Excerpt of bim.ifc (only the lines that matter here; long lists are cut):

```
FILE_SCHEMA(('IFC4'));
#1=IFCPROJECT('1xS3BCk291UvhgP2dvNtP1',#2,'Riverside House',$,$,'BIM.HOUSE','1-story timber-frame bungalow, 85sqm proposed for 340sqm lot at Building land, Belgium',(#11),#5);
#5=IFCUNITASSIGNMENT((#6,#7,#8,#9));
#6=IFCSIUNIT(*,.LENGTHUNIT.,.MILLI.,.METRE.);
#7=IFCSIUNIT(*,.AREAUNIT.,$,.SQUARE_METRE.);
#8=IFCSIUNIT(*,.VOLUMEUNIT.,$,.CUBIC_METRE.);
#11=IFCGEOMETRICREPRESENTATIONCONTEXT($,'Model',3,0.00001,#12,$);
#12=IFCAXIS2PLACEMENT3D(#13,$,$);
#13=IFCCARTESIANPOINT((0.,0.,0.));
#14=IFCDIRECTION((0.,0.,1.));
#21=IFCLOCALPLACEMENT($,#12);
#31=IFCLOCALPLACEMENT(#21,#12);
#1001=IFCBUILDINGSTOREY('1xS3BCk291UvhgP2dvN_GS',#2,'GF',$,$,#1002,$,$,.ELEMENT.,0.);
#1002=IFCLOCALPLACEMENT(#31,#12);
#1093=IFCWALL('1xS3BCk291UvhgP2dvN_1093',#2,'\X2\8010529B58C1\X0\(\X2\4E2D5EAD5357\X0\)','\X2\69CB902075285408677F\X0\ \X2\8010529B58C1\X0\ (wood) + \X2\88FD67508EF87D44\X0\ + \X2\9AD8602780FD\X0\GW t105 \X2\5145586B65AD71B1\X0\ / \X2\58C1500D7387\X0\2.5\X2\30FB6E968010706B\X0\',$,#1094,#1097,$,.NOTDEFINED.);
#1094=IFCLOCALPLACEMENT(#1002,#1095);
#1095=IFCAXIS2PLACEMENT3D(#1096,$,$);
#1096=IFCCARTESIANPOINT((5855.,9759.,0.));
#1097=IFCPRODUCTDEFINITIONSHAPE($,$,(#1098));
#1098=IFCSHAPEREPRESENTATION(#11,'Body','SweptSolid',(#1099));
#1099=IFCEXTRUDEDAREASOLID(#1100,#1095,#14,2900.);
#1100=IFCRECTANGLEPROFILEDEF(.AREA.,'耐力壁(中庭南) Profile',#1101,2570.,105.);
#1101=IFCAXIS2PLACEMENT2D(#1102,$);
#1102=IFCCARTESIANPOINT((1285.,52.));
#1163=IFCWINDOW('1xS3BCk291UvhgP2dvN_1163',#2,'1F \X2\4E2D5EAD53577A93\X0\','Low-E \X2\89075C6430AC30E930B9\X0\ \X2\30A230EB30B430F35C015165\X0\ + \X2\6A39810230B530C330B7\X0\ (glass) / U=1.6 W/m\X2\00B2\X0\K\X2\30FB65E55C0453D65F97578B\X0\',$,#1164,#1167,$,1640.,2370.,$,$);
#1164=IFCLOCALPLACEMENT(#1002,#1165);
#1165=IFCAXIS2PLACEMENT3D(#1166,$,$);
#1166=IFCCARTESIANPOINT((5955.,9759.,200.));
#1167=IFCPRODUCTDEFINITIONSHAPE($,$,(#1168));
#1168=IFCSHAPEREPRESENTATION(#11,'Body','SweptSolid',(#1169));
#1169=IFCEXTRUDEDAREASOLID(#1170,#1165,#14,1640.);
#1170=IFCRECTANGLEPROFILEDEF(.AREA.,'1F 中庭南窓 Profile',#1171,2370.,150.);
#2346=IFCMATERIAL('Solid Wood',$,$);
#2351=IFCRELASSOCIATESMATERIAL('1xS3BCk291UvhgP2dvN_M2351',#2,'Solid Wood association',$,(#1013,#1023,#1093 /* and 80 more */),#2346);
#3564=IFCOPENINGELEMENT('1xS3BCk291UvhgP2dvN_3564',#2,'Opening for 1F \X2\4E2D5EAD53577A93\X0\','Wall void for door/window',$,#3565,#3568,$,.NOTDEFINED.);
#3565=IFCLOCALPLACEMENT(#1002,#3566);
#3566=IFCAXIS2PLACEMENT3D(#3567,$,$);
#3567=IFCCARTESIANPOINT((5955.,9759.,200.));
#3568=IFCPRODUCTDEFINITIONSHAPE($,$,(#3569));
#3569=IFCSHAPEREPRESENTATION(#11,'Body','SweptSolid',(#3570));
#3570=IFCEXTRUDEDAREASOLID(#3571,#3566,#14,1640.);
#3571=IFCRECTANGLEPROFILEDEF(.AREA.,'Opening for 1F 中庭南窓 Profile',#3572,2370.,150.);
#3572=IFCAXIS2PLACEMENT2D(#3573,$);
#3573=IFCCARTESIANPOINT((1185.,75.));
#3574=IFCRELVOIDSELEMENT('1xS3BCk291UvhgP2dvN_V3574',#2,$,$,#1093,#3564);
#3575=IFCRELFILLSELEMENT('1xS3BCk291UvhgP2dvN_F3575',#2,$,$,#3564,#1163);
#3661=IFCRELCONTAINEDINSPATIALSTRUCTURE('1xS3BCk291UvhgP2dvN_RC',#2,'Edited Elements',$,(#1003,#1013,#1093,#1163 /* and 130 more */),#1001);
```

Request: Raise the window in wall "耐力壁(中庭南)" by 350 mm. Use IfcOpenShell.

```python
import numpy as np
import ifcopenshell
import ifcopenshell.api.geometry
import ifcopenshell.util.placement
import ifcopenshell.util.unit

model = ifcopenshell.open("bim.ifc")
unit_scale = ifcopenshell.util.unit.calculate_unit_scale(model)

window = model.by_guid("1xS3BCk291UvhgP2dvN_1163")
opening = window.FillsVoids[0].RelatingOpeningElement
dz = 0.35 / unit_scale

shift = np.array([0.0, 0.0, dz])
# The window is not placed relative to its opening, so move both.
for product in (opening, window):
    matrix = ifcopenshell.util.placement.get_local_placement(product.ObjectPlacement)
    matrix[:3, 3] += shift
    ifcopenshell.api.geometry.edit_object_placement(model, product=product, matrix=matrix, is_si=False)

print(f"moved by {dz * unit_scale:+.3f} m")

model.write("bim_edited.ifc")
```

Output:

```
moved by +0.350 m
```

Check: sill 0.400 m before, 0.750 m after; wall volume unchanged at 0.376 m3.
